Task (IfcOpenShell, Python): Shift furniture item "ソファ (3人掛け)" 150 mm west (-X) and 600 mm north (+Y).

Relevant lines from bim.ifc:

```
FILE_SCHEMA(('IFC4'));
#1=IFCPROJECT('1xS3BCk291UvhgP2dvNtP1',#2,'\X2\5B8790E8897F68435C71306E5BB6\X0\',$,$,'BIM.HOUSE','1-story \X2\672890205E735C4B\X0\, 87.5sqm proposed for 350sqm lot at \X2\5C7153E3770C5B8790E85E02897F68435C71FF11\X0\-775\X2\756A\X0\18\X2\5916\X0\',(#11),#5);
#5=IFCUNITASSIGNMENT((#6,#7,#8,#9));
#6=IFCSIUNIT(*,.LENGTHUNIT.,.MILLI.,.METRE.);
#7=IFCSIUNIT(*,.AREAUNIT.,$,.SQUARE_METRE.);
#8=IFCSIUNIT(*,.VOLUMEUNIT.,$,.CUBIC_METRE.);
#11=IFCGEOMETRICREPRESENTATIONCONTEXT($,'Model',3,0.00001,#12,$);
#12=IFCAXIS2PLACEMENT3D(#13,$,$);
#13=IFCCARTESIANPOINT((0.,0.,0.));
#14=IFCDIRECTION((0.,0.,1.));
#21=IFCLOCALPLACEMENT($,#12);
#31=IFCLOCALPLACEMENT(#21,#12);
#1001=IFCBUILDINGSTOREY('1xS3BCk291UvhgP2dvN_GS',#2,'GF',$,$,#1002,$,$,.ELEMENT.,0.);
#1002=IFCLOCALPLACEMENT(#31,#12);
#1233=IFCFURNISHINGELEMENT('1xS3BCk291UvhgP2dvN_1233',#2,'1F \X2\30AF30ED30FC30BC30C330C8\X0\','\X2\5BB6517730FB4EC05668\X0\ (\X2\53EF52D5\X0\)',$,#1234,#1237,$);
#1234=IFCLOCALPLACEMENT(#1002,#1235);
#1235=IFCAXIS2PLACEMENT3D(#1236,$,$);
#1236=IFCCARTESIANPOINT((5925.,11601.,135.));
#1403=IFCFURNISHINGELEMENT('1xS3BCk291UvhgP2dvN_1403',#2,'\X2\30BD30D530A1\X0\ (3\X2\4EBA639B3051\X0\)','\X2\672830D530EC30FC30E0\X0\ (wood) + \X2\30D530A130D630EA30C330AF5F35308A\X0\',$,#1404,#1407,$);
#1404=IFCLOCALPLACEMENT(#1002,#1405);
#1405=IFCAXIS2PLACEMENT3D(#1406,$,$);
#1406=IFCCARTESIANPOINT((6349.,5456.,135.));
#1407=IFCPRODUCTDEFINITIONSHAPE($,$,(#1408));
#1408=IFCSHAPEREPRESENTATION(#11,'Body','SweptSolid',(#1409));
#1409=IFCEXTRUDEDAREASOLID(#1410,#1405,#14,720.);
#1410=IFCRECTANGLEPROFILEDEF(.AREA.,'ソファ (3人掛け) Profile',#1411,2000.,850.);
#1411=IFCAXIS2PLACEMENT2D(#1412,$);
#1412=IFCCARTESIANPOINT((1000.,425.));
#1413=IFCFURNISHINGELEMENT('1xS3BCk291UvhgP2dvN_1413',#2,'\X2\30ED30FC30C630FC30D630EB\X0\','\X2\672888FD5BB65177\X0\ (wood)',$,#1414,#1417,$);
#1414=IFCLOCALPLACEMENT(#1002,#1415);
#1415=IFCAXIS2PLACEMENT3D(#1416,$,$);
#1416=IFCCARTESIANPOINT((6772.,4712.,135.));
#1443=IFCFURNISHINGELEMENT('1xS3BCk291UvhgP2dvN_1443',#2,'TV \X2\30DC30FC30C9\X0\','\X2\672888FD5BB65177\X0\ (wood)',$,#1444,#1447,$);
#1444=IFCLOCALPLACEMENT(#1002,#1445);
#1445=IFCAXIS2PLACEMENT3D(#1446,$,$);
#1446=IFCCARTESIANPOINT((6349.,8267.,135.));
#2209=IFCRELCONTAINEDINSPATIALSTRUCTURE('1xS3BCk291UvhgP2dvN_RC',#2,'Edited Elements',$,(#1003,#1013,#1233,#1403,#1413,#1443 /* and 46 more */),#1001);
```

```python
import ifcopenshell
import ifcopenshell.api.geometry
import ifcopenshell.util.placement
import ifcopenshell.util.unit

model = ifcopenshell.open("bim.ifc")
unit_scale = ifcopenshell.util.unit.calculate_unit_scale(model)

item = model.by_guid("1xS3BCk291UvhgP2dvN_1403")
matrix = ifcopenshell.util.placement.get_local_placement(item.ObjectPlacement)
matrix[0, 3] -= 0.15 / unit_scale
matrix[1, 3] += 0.6 / unit_scale
ifcopenshell.api.geometry.edit_object_placement(model, product=item, matrix=matrix, is_si=False)

print(ifcopenshell.util.placement.get_local_placement(item.ObjectPlacement).round(3) + 0.0)

model.write("bim_edited.ifc")
```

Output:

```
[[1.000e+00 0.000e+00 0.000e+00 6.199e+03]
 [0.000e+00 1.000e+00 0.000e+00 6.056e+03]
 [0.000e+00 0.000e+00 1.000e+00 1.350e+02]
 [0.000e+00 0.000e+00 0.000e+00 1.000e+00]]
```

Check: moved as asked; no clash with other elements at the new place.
